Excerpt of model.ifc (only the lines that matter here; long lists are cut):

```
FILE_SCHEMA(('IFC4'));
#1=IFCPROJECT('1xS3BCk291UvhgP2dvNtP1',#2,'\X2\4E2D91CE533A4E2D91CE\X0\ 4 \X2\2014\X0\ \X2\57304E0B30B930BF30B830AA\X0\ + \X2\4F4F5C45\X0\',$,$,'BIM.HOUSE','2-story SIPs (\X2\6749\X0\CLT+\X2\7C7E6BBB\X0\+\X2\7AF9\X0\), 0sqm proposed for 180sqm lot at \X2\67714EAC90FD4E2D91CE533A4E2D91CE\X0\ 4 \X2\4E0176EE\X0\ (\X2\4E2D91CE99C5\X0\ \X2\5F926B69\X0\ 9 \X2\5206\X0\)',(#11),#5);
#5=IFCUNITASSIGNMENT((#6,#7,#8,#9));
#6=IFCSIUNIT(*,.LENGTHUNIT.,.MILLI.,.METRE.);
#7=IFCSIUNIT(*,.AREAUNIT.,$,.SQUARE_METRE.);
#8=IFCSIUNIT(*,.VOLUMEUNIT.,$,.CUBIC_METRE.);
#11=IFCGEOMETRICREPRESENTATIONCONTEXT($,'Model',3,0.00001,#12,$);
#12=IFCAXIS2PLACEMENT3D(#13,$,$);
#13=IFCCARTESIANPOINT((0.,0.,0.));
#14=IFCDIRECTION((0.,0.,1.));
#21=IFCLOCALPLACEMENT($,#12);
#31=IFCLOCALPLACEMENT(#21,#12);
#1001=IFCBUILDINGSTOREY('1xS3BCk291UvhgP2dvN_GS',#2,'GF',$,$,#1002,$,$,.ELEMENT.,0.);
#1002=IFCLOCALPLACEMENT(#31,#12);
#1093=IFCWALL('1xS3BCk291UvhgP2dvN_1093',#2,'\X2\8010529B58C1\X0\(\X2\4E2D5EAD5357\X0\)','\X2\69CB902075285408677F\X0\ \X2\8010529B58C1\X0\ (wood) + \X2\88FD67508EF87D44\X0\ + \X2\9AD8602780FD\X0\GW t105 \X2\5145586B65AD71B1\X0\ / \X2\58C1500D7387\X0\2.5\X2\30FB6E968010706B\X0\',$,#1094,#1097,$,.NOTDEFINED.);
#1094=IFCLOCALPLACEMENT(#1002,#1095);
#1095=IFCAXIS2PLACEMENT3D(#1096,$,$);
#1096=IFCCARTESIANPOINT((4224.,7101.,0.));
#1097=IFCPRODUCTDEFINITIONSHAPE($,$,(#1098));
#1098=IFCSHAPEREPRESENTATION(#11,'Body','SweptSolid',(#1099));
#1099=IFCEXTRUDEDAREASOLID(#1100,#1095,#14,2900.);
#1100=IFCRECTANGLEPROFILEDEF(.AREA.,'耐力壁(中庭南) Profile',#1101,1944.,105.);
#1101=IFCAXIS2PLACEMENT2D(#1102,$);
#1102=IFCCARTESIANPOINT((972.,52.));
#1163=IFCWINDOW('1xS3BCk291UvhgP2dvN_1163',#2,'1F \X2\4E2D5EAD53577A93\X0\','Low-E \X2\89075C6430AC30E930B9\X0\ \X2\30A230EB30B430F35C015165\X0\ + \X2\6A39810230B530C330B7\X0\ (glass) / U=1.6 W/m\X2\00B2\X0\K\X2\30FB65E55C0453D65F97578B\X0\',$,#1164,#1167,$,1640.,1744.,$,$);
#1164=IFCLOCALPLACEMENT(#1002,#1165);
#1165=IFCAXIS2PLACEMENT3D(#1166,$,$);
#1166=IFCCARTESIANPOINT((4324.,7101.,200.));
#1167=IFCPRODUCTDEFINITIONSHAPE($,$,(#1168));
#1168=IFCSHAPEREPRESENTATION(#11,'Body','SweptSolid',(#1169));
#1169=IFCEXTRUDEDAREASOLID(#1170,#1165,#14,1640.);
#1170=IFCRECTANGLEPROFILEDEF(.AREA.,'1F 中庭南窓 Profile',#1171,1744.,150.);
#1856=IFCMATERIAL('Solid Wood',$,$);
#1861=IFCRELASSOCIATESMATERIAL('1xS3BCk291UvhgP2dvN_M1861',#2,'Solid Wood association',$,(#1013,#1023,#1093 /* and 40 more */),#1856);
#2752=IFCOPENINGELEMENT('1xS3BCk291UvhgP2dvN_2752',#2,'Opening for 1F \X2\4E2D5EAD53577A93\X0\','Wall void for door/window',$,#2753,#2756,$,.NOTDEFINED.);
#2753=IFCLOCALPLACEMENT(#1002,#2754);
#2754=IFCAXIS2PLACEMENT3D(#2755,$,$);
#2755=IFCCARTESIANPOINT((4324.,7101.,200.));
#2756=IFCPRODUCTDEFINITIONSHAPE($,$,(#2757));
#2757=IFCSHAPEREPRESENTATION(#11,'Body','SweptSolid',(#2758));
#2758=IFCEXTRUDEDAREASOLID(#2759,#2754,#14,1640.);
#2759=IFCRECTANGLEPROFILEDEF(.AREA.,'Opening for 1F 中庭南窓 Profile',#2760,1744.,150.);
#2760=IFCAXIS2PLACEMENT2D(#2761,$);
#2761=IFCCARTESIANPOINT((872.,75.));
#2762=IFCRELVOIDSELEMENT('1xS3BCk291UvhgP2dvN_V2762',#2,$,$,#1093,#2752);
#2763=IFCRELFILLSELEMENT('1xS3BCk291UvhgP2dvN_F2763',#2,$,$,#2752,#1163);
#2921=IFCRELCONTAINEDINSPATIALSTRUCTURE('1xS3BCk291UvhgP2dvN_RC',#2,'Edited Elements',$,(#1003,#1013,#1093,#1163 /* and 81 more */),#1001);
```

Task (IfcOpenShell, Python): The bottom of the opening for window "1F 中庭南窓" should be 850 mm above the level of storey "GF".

```python
import numpy as np
import ifcopenshell
import ifcopenshell.api.geometry
import ifcopenshell.geom
import ifcopenshell.util.element
import ifcopenshell.util.placement
import ifcopenshell.util.shape
import ifcopenshell.util.unit

model = ifcopenshell.open("model.ifc")
unit_scale = ifcopenshell.util.unit.calculate_unit_scale(model)

window = model.by_guid("1xS3BCk291UvhgP2dvN_1163")
opening = window.FillsVoids[0].RelatingOpeningElement
storey = ifcopenshell.util.element.get_container(window, ifc_class="IfcBuildingStorey")
level = ifcopenshell.util.placement.get_local_placement(storey.ObjectPlacement)[2, 3]

# The opening's origin need not be at the sill, so measure its lowest point.
shape = ifcopenshell.geom.create_shape(ifcopenshell.geom.settings(), opening)
bottom = ifcopenshell.util.shape.get_shape_bottom_elevation(shape, shape.geometry) / unit_scale
dz = level + 0.85 / unit_scale - bottom

shift = np.array([0.0, 0.0, dz])
# The window is not placed relative to its opening, so move both.
for product in (opening, window):
    matrix = ifcopenshell.util.placement.get_local_placement(product.ObjectPlacement)
    matrix[:3, 3] += shift
    ifcopenshell.api.geometry.edit_object_placement(model, product=product, matrix=matrix, is_si=False)

print(f"moved by {dz * unit_scale:+.3f} m")

model.write("model_edited.ifc")
```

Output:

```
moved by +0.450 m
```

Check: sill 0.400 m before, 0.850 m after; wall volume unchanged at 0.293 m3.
